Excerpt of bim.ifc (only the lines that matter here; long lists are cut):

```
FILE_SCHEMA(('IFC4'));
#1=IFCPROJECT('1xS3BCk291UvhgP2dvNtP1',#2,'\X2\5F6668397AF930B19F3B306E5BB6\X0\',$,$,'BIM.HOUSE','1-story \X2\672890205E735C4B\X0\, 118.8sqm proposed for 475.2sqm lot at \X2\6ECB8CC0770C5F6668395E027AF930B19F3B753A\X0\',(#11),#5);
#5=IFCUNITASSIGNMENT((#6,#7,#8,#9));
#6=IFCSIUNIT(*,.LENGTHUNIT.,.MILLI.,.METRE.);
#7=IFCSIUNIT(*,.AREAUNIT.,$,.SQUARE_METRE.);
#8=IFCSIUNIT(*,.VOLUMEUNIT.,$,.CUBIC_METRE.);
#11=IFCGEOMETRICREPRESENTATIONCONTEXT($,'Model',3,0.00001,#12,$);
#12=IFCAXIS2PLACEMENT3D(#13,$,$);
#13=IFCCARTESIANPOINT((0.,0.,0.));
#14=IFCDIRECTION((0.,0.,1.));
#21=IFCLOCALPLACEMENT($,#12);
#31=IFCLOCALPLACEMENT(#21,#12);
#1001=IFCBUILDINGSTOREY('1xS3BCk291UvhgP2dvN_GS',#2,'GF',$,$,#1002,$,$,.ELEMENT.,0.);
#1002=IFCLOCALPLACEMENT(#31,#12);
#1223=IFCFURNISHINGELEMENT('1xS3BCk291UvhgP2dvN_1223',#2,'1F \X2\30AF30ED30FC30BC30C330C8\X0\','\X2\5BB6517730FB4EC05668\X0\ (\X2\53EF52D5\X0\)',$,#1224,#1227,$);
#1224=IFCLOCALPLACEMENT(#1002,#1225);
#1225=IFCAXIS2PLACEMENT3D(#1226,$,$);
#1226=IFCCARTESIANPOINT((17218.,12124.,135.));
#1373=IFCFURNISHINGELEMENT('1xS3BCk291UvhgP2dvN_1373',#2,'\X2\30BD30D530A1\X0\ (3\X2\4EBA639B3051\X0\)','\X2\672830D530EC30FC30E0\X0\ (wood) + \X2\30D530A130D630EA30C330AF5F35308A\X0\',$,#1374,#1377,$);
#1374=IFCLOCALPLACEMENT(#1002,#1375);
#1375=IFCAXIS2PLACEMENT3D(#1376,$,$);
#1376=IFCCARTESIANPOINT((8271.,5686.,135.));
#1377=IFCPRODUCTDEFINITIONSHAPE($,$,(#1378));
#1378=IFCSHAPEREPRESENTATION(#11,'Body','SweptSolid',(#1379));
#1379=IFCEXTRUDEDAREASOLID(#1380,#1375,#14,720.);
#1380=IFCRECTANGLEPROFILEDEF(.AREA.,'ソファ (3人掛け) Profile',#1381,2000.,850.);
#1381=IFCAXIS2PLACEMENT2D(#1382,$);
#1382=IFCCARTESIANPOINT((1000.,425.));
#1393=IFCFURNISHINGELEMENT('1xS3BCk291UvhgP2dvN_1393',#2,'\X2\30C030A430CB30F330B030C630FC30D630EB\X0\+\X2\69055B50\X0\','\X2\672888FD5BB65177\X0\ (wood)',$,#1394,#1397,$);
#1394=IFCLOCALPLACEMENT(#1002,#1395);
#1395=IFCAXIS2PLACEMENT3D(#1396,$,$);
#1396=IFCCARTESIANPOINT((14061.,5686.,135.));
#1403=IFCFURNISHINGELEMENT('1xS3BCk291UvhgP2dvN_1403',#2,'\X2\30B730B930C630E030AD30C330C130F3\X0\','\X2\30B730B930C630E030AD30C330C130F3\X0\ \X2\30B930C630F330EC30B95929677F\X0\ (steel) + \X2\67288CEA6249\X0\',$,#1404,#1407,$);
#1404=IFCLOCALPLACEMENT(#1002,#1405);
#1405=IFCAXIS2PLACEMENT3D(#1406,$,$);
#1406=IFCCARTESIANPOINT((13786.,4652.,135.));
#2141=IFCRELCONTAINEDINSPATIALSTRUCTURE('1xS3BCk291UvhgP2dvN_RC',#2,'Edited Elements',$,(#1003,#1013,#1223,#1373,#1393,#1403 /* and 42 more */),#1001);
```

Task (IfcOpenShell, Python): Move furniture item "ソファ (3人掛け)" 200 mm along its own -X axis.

```python
import ifcopenshell
import ifcopenshell.api.geometry
import ifcopenshell.util.placement

model = ifcopenshell.open("bim.ifc")

item = model.by_id(1373)
matrix = ifcopenshell.util.placement.get_local_placement(item.ObjectPlacement)
matrix[:3, 3] -= matrix[:3, 0] * 200.0
ifcopenshell.api.geometry.edit_object_placement(model, product=item, matrix=matrix, is_si=False)

print(ifcopenshell.util.placement.get_local_placement(item.ObjectPlacement).round(3) + 0.0)

model.write("bim_v2.ifc")
```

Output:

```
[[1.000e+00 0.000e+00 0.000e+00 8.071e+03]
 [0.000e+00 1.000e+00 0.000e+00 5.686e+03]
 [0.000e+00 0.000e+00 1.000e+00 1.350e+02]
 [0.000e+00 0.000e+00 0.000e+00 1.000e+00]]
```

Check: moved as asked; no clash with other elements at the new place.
